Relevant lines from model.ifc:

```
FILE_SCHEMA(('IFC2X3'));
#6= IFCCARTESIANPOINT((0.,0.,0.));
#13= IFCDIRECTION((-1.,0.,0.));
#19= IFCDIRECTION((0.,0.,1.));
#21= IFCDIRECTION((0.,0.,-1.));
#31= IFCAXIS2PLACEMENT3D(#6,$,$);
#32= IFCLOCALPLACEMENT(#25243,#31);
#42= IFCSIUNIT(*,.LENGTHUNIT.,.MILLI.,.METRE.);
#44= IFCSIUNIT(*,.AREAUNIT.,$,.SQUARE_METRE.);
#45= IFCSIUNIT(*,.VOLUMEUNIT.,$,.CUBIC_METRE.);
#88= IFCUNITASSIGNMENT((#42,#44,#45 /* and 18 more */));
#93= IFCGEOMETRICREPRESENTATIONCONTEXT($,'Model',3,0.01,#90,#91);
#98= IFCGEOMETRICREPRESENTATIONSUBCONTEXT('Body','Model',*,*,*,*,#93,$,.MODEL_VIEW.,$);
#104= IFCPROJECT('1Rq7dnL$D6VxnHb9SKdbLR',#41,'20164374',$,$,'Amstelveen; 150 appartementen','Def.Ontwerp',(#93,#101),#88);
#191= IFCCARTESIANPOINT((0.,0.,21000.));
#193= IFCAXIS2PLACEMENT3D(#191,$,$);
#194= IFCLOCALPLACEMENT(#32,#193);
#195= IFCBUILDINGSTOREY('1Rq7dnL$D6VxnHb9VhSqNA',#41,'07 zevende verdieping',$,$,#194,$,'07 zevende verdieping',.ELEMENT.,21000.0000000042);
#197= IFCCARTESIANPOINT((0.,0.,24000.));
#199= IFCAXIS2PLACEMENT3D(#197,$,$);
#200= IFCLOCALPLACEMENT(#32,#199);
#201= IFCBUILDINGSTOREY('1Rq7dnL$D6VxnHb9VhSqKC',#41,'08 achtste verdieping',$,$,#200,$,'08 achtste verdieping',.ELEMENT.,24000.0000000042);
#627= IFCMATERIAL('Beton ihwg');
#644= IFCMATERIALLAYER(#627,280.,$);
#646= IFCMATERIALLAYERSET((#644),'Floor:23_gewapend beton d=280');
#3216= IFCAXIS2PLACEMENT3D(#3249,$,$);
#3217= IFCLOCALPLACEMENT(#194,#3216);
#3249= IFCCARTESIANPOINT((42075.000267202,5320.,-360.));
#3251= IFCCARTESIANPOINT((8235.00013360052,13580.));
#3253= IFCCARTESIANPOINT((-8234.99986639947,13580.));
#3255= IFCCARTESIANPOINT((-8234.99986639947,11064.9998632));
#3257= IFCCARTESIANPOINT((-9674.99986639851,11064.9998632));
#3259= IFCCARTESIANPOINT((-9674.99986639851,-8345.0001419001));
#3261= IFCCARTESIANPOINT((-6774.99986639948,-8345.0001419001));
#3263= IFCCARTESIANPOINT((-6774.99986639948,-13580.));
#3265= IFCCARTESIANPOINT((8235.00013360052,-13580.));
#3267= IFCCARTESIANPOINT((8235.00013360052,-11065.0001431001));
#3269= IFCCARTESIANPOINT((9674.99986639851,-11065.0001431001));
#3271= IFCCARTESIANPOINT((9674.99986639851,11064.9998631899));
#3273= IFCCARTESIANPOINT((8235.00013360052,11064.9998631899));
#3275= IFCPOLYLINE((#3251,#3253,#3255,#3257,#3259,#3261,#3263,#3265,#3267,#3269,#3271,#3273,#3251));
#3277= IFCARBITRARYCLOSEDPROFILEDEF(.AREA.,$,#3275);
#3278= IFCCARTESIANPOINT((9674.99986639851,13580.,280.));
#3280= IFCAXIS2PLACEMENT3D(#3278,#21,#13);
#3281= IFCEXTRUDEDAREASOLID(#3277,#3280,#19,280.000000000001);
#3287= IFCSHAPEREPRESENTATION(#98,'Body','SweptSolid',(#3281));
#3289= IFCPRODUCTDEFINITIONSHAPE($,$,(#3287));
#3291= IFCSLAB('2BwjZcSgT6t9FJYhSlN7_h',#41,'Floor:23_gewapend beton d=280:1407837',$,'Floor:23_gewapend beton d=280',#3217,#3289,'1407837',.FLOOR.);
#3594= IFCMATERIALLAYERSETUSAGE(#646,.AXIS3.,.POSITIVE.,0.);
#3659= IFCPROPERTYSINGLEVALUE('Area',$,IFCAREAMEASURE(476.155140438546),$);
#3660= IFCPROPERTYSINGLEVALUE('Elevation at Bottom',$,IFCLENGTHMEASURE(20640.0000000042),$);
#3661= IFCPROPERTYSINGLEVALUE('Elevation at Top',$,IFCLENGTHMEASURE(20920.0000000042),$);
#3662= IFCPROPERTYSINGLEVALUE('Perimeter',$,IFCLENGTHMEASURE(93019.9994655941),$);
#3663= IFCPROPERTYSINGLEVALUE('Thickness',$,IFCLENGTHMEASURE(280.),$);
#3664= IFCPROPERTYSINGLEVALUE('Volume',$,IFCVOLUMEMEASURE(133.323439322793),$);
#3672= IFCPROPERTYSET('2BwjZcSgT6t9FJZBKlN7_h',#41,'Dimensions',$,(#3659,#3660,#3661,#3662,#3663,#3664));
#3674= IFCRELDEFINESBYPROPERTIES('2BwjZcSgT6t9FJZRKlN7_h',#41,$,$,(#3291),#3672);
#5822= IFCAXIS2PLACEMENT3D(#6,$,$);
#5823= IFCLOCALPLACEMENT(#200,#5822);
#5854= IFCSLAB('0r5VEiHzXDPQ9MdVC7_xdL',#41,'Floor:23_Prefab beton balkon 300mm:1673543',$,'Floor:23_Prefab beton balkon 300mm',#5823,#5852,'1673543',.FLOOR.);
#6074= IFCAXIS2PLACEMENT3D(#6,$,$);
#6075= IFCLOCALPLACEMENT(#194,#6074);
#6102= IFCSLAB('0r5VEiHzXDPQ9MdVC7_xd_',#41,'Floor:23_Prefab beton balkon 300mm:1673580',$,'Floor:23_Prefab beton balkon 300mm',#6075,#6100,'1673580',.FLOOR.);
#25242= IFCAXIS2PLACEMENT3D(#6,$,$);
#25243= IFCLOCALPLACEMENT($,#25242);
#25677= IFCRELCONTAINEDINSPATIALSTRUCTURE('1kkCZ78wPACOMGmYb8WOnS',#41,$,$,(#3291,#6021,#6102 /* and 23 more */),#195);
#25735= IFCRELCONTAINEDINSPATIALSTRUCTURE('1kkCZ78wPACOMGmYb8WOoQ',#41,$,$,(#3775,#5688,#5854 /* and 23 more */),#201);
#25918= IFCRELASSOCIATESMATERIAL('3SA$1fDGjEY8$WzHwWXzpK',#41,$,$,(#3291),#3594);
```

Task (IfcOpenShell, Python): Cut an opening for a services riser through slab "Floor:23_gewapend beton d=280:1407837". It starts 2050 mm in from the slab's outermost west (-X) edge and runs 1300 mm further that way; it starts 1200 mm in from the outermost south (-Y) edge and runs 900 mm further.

```python
import numpy as np
import ifcopenshell
import ifcopenshell.api.feature
import ifcopenshell.api.geometry
import ifcopenshell.api.pset
import ifcopenshell.api.root
import ifcopenshell.geom
import ifcopenshell.util.element
import ifcopenshell.util.placement
import ifcopenshell.util.representation
import ifcopenshell.util.shape
import ifcopenshell.util.unit

model = ifcopenshell.open("model.ifc")
unit_scale = ifcopenshell.util.unit.calculate_unit_scale(model)
area_scale = ifcopenshell.util.unit.calculate_unit_scale(model, "AREAUNIT")
volume_scale = ifcopenshell.util.unit.calculate_unit_scale(model, "VOLUMEUNIT")
settings = ifcopenshell.geom.settings()


def volume(element):
    """Net volume in cubic metres, openings subtracted."""
    shape = ifcopenshell.geom.create_shape(settings, element)
    return ifcopenshell.util.shape.get_volume(shape.geometry)


slab = model.by_guid("2BwjZcSgT6t9FJYhSlN7_h")
before = volume(slab)

# Extent in the slab's own axes, in metres. The edges named are its -X and -Y sides.
slab_shape = ifcopenshell.geom.create_shape(settings, slab)
vertices = ifcopenshell.util.shape.get_vertices(slab_shape.geometry)
x_min, y_min, bottom = vertices.min(axis=0)
top = vertices[:, 2].max()

opening = ifcopenshell.api.root.create_entity(model, ifc_class="IfcOpeningElement", name="Services riser opening")
context = ifcopenshell.util.representation.get_context(model, "Model", "Body", "MODEL_VIEW")
width, depth = 1.3, 0.9
outline = [(0.0, 0.0), (width, 0.0), (width, depth), (0.0, depth), (0.0, 0.0)]
# Overshoot both faces by 50 mm so the cut is clean.
shape = ifcopenshell.api.geometry.add_slab_representation(
    model, context=context, depth=top - bottom + 0.1, polyline=outline
)
ifcopenshell.api.geometry.assign_representation(model, product=opening, representation=shape)

matrix = ifcopenshell.util.placement.get_local_placement(slab.ObjectPlacement)
matrix[:, 3] = matrix @ np.append(np.array([x_min + 2.05, y_min + 1.2, bottom - 0.05]) / unit_scale, 1.0)
ifcopenshell.api.geometry.edit_object_placement(model, product=opening, matrix=matrix, is_si=False)
ifcopenshell.api.feature.add_feature(model, feature=opening, element=slab)

after = volume(slab)

# Update the slab's stored quantities.
pset = model.by_id(ifcopenshell.util.element.get_pset(slab, "Dimensions", should_inherit=False)["id"])
ifcopenshell.api.pset.edit_pset(model, pset=pset, properties={
    "Area": model.create_entity("IfcAreaMeasure", after / (top - bottom) / area_scale),
    "Volume": model.create_entity("IfcVolumeMeasure", after / volume_scale),
})

print(f"slab volume {before:.3f} -> {after:.3f} m3")

model.write("model_edited.ifc")
```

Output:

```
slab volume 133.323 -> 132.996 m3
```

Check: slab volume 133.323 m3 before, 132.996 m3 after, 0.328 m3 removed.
